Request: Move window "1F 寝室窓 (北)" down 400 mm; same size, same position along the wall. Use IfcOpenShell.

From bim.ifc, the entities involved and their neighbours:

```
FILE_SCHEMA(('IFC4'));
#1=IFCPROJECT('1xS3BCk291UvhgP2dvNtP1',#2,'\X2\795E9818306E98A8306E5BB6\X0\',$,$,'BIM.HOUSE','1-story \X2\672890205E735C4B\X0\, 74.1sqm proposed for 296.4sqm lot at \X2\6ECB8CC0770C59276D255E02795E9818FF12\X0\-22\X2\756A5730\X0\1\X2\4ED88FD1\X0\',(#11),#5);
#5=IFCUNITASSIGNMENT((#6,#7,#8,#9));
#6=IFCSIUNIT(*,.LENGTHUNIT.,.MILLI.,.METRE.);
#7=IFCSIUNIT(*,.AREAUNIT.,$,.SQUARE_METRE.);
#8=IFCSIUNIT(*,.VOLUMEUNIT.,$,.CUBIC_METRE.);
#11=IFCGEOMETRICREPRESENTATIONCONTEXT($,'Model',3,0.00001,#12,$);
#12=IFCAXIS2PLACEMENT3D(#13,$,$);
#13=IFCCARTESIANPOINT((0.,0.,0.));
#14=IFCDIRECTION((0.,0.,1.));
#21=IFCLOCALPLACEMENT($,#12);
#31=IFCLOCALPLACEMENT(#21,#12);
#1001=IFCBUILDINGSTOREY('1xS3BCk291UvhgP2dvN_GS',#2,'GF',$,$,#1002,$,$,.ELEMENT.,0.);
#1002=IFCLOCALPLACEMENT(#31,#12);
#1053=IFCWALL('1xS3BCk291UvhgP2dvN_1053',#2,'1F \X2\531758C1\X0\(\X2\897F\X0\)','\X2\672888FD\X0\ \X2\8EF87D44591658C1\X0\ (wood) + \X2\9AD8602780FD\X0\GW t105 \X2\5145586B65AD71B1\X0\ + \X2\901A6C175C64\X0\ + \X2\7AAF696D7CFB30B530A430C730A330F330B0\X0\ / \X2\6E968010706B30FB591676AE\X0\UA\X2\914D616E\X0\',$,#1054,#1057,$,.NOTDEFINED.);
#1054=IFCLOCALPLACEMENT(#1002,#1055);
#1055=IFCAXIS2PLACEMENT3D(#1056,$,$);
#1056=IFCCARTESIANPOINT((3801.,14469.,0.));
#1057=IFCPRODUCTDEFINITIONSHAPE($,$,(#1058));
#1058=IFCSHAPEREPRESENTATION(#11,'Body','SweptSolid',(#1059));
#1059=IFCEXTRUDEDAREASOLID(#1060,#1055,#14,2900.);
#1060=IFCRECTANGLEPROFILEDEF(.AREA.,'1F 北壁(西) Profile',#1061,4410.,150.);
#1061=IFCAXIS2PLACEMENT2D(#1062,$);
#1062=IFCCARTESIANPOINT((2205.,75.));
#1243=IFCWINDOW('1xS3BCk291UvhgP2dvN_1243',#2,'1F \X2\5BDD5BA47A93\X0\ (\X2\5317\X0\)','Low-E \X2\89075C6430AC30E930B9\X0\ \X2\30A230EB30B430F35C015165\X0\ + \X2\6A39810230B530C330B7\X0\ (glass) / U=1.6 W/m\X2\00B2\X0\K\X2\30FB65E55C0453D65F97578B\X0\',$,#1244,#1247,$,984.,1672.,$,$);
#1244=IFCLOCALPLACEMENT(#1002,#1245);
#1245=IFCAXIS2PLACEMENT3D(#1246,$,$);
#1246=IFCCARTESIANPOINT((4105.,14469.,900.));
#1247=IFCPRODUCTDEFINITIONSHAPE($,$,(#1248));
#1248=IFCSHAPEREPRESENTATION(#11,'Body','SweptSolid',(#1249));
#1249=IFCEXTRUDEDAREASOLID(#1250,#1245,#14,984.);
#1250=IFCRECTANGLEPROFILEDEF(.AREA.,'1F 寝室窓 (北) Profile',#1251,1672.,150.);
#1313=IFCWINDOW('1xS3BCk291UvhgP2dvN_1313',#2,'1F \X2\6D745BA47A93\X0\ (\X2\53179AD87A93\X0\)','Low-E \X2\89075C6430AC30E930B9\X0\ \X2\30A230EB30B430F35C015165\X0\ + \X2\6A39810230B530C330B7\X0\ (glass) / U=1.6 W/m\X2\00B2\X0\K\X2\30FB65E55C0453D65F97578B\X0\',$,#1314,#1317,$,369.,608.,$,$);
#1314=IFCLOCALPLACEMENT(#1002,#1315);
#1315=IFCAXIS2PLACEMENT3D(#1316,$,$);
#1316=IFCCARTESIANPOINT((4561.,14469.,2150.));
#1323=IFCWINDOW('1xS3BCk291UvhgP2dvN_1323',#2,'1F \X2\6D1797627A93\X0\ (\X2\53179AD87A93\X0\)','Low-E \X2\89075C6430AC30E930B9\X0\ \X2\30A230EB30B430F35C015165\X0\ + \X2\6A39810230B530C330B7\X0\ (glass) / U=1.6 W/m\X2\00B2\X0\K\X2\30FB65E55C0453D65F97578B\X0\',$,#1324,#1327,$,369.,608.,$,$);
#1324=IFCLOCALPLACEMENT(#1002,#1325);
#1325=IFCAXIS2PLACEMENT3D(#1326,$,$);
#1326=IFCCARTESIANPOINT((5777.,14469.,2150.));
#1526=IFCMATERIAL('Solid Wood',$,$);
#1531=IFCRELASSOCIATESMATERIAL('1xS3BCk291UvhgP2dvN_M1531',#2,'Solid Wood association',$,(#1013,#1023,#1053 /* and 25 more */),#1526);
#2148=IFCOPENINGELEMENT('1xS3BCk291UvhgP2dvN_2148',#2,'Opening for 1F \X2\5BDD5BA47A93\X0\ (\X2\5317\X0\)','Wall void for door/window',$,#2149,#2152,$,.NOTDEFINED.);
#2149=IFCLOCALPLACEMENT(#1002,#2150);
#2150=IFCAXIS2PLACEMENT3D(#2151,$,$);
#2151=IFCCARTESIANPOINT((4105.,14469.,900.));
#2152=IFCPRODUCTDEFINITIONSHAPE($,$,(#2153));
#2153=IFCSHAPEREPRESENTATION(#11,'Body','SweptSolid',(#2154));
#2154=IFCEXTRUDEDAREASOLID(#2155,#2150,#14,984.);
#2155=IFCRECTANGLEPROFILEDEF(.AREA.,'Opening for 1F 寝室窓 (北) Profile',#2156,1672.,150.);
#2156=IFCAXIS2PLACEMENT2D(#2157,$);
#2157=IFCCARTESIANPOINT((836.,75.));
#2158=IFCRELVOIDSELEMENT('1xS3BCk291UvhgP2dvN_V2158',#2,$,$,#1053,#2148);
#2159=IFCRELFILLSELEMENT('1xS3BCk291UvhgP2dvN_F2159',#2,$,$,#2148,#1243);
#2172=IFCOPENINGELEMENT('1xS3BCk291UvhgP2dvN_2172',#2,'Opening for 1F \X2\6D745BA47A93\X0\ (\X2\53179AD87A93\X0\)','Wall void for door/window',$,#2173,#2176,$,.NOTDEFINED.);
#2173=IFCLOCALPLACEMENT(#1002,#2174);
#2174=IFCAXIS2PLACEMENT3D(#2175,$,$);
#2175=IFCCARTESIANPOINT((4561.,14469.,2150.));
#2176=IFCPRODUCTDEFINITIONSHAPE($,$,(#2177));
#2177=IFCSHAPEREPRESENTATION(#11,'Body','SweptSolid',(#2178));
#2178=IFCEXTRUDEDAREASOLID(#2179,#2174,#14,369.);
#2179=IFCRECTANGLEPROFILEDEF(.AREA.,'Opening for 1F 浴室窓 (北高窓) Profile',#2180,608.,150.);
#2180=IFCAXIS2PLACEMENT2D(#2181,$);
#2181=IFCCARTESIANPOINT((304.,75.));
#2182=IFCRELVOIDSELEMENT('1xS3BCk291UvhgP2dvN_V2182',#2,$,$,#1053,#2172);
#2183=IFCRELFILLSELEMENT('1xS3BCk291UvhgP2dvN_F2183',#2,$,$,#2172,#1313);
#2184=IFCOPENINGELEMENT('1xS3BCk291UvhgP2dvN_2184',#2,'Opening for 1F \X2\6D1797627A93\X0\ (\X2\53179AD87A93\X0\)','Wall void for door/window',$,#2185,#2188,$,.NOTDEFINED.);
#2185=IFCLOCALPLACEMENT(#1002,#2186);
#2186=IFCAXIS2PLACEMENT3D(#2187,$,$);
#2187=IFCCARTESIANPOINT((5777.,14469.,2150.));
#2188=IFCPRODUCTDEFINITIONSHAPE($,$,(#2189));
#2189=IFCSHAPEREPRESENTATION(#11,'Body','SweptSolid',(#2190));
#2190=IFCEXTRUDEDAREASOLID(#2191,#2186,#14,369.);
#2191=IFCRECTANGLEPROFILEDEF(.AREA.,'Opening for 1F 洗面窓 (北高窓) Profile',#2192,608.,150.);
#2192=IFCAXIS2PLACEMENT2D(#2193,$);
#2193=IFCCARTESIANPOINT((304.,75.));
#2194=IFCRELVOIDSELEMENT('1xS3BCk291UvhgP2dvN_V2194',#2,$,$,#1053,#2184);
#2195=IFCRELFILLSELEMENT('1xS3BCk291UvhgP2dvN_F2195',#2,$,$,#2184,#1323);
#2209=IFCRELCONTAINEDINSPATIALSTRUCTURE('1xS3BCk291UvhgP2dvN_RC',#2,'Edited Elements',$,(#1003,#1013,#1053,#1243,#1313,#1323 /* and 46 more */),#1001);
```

```python
import numpy as np
import ifcopenshell
import ifcopenshell.api.geometry
import ifcopenshell.util.placement
import ifcopenshell.util.unit

model = ifcopenshell.open("bim.ifc")
unit_scale = ifcopenshell.util.unit.calculate_unit_scale(model)

window = model.by_guid("1xS3BCk291UvhgP2dvN_1243")
opening = window.FillsVoids[0].RelatingOpeningElement
dz = -400.0

shift = np.array([0.0, 0.0, dz])
# The window is not placed relative to its opening, so move both.
for product in (opening, window):
    matrix = ifcopenshell.util.placement.get_local_placement(product.ObjectPlacement)
    matrix[:3, 3] += shift
    ifcopenshell.api.geometry.edit_object_placement(model, product=product, matrix=matrix, is_si=False)

print(f"moved by {dz * unit_scale:+.3f} m")

model.write("bim_v2.ifc")
```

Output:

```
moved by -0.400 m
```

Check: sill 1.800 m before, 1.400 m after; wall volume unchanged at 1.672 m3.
